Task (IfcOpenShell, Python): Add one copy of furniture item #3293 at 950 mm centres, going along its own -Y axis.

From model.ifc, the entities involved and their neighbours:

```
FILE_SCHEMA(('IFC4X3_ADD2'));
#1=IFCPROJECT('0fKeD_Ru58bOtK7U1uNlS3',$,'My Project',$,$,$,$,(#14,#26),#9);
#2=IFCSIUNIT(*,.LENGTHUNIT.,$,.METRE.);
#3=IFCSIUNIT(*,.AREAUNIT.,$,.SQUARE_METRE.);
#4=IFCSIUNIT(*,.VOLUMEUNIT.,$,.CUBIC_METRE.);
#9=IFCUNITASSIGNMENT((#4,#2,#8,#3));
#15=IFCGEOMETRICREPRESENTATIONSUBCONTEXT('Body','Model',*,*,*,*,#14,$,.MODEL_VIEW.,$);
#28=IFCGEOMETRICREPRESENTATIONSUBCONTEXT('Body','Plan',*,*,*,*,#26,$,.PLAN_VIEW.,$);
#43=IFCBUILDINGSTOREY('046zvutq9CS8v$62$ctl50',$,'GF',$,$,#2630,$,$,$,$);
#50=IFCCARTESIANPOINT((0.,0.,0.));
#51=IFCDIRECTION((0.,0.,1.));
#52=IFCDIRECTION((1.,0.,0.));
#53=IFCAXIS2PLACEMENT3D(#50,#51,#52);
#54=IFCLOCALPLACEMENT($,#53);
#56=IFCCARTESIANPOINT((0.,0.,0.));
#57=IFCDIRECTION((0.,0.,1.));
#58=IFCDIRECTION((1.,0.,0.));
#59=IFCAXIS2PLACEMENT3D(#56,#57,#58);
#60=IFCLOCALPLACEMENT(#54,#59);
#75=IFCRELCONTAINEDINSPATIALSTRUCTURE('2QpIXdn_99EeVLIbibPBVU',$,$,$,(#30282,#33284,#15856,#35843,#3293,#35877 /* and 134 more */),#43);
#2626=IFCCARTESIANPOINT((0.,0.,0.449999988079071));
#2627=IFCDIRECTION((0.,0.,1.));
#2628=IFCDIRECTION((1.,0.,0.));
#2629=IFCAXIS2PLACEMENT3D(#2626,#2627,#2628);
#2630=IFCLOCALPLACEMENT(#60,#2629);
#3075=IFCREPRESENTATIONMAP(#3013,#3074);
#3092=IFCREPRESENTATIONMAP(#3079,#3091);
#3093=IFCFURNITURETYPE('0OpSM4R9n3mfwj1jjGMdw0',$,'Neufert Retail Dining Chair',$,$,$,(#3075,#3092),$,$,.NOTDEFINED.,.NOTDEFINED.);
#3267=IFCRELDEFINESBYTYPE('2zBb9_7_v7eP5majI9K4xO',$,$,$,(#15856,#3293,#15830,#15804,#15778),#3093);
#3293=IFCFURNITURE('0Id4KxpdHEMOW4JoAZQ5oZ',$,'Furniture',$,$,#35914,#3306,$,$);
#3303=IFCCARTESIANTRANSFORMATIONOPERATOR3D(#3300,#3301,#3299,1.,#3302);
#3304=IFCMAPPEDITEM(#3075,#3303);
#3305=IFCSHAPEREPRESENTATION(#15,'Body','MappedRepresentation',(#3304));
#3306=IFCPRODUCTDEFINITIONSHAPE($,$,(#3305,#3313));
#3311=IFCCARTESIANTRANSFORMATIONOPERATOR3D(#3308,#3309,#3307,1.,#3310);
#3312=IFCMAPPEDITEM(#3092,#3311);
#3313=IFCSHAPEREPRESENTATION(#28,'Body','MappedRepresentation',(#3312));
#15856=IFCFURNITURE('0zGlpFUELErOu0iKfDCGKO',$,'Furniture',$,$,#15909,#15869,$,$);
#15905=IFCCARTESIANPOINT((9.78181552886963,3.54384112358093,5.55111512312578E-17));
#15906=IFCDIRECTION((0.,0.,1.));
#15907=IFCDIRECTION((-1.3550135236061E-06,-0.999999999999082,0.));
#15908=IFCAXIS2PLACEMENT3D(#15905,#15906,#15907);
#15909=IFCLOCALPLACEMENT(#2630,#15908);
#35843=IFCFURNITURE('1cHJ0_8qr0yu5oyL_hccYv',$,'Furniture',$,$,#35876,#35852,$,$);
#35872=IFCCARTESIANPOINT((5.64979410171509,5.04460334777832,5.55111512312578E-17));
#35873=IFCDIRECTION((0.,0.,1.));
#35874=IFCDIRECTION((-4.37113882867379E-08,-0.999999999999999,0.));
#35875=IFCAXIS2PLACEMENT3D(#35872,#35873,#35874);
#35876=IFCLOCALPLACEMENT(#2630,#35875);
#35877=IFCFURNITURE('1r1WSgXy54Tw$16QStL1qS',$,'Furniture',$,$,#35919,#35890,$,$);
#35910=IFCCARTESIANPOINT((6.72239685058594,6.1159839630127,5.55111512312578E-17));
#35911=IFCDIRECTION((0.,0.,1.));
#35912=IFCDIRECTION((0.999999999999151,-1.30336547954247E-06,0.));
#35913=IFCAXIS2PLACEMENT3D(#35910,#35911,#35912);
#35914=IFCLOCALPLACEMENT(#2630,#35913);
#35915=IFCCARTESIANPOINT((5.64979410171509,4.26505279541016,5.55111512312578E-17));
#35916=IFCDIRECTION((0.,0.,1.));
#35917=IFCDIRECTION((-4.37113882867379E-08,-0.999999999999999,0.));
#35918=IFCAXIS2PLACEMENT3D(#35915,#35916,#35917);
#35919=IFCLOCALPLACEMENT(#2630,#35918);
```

```python
import ifcopenshell
import ifcopenshell.api.geometry
import ifcopenshell.api.root
import ifcopenshell.util.element
import ifcopenshell.util.placement
import ifcopenshell.util.unit

model = ifcopenshell.open("model.ifc")
unit_scale = ifcopenshell.util.unit.calculate_unit_scale(model)

source = model.by_guid("0Id4KxpdHEMOW4JoAZQ5oZ")
base = ifcopenshell.util.placement.get_local_placement(source.ObjectPlacement)
step = -base[:3, 1] * 0.95 / unit_scale

for i in range(1, 2):
    copy = ifcopenshell.api.root.copy_class(model, product=source)
    copy.Representation = ifcopenshell.util.element.copy_deep(
        model, source.Representation, exclude=["IfcGeometricRepresentationContext", "IfcRepresentationMap"]
    )
    matrix = base.copy()
    matrix[:3, 3] += i * step
    print("added at", matrix[:3, 3].round(3) + 0.0)
    ifcopenshell.api.geometry.edit_object_placement(model, product=copy, matrix=matrix, is_si=False)

model.write("model_updated.ifc")
```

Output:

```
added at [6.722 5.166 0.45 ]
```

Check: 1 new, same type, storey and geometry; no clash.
